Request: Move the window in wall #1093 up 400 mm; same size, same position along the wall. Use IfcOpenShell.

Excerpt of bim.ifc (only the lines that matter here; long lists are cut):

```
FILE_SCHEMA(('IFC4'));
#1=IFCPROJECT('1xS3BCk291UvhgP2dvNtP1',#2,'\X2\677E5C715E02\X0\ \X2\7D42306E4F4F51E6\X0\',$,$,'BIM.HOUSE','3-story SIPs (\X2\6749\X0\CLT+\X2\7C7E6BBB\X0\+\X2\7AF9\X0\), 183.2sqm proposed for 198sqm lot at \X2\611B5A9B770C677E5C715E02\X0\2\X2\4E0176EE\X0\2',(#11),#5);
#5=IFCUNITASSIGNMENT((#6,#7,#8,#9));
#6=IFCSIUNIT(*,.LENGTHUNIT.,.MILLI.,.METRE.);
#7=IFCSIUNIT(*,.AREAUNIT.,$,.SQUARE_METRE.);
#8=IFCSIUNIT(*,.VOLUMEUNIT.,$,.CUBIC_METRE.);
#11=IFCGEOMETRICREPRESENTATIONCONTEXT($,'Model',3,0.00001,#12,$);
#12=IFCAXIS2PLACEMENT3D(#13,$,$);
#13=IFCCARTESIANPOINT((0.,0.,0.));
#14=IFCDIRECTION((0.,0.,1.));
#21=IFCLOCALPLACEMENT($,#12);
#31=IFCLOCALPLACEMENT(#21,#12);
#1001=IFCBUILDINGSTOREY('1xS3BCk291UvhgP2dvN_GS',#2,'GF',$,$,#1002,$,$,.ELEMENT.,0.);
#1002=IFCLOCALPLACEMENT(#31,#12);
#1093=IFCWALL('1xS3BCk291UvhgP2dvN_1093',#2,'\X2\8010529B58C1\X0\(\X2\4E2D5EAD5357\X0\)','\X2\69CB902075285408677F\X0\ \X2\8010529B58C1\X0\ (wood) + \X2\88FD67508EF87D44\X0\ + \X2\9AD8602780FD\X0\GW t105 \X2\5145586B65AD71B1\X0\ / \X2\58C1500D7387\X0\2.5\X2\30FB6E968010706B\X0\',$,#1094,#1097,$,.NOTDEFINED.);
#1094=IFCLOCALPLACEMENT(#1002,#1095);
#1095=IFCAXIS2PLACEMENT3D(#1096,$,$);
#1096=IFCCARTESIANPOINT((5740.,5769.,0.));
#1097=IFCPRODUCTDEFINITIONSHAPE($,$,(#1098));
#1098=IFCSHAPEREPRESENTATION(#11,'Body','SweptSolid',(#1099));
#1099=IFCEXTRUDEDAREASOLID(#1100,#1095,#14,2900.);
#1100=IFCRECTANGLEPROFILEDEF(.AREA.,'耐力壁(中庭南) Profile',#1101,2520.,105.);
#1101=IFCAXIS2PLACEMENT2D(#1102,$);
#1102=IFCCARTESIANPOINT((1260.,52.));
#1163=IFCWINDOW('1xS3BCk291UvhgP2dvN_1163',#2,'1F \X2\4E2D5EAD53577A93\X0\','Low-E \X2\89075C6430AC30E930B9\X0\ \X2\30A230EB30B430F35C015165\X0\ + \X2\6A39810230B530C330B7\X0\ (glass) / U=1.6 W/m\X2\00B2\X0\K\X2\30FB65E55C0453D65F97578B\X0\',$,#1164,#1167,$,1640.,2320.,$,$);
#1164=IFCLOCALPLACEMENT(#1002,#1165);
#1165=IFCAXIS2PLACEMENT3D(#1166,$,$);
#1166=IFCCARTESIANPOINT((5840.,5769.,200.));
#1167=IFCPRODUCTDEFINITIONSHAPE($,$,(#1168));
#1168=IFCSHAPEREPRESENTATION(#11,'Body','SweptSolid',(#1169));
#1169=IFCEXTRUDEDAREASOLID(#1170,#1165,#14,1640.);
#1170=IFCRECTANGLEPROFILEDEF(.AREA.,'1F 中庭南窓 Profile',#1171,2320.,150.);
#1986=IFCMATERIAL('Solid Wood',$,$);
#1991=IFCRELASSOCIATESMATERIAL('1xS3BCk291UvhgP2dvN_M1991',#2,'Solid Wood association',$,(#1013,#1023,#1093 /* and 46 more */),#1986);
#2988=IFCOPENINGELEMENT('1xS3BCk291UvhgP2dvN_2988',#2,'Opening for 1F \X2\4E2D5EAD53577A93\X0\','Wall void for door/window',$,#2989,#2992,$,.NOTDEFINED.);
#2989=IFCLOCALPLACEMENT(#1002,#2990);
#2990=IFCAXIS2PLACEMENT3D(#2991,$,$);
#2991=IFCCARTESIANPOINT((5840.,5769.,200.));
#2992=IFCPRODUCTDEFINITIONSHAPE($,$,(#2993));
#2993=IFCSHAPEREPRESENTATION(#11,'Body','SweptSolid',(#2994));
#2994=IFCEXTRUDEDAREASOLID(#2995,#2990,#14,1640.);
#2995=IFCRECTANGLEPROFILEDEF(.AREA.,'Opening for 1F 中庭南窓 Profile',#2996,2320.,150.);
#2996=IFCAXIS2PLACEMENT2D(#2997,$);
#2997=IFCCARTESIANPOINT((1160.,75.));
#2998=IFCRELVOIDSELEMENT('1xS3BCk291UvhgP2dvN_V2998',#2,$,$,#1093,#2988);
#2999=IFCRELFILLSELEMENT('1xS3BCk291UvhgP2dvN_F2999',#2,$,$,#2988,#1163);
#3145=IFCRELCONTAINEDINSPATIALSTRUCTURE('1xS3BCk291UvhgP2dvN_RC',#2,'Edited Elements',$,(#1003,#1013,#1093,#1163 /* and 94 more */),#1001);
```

```python
import numpy as np
import ifcopenshell
import ifcopenshell.api.geometry
import ifcopenshell.util.placement
import ifcopenshell.util.unit

model = ifcopenshell.open("bim.ifc")
unit_scale = ifcopenshell.util.unit.calculate_unit_scale(model)

window = model.by_guid("1xS3BCk291UvhgP2dvN_1163")
opening = window.FillsVoids[0].RelatingOpeningElement
dz = 400.0

shift = np.array([0.0, 0.0, dz])
# The window is not placed relative to its opening, so move both.
for product in (opening, window):
    matrix = ifcopenshell.util.placement.get_local_placement(product.ObjectPlacement)
    matrix[:3, 3] += shift
    ifcopenshell.api.geometry.edit_object_placement(model, product=product, matrix=matrix, is_si=False)

print(f"moved by {dz * unit_scale:+.3f} m")

model.write("bim_v2.ifc")
```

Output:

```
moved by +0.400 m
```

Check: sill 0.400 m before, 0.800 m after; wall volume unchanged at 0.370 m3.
